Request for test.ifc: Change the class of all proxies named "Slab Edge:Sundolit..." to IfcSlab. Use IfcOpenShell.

First a look at what the model holds.

```python
import re

import ifcopenshell

model = ifcopenshell.open("test.ifc")
print(model.schema)
seen = {}
for e in model.by_type("IfcBuildingElementProxy"):
    name = re.sub(r":\d+(:\d+)?$", "", e.Name or "")  # drop the element id that some exporters append
    seen[name] = seen.get(name, 0) + 1
for name, count in sorted(seen.items()):
    print(count, "x", name)
```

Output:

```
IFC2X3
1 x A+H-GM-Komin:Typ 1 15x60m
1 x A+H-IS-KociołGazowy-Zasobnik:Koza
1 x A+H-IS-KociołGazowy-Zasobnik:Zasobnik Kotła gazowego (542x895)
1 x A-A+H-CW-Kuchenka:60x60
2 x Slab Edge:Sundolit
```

```python
import ifcopenshell
import ifcopenshell.api.root

model = ifcopenshell.open("test.ifc")

proxies = [e.id() for e in model.by_type("IfcBuildingElementProxy") if (e.Name or "").startswith("Slab Edge:Sundolit")]
for step_id in proxies:
    proxy = model.by_id(step_id)
    ifcopenshell.api.root.reassign_class(model, product=proxy, ifc_class="IfcSlab", predefined_type="FLOOR")

print(sum(model.by_id(i).is_a("IfcSlab") for i in proxies), "reclassified")

model.write("test_updated.ifc")
```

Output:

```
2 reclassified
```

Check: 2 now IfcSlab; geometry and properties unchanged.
